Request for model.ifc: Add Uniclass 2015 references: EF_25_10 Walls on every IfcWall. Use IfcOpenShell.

First a look at what the model holds.

```python
import ifcopenshell

model = ifcopenshell.open("model.ifc")
print(model.schema)
print("classifications:", [c.Name for c in model.by_type("IfcClassification")])
for ifc_class in ("IfcDoor", "IfcRoof", "IfcStair", "IfcWall", "IfcWindow"):
    print(ifc_class, len(model.by_type(ifc_class)))
```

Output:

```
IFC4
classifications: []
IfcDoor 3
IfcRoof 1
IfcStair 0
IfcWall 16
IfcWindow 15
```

```python
import ifcopenshell
import ifcopenshell.api.classification

model = ifcopenshell.open("model.ifc")

system = ifcopenshell.api.classification.add_classification(model, classification="Uniclass 2015")

codes = {
    "IfcWall": ("EF_25_10", "Walls"),
}
for ifc_class, (code, name) in codes.items():
    products = model.by_type(ifc_class)
    ifcopenshell.api.classification.add_reference(
        model, products=products, classification=system, identification=code, name=name
    )
    print(code, len(products))

model.write("model_updated.ifc")
```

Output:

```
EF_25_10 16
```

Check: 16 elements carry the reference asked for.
